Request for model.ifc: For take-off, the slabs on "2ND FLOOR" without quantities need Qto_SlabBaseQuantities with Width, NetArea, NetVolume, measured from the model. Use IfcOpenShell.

First a look at what the model holds.

```python
import ifcopenshell
import ifcopenshell.util.element
import ifcopenshell.util.unit

model = ifcopenshell.open("model.ifc")
print(model.schema)
for unit_type in ("LENGTHUNIT", "AREAUNIT", "VOLUMEUNIT"):
    print(unit_type, ifcopenshell.util.unit.calculate_unit_scale(model, unit_type))
storey = next(s for s in model.by_type("IfcBuildingStorey") if s.Name == "2ND FLOOR")
slabs = [e for e in ifcopenshell.util.element.get_decomposition(storey) if e.is_a("IfcSlab")]
for e in sorted(slabs, key=lambda e: e.id()):
    print(e.id(), e.is_a(), e.Name, list(ifcopenshell.util.element.get_psets(e, qtos_only=True)), sep=" | ")
```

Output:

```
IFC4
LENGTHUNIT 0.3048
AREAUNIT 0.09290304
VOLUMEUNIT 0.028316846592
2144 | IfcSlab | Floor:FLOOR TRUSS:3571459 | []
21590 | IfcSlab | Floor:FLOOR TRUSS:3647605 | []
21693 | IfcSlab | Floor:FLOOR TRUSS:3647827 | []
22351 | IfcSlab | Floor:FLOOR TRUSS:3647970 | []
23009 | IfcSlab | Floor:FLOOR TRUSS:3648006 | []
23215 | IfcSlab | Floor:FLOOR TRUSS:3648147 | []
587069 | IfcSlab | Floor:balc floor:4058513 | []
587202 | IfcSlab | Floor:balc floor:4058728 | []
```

```python
import ifcopenshell
import ifcopenshell.api.pset
import ifcopenshell.geom
import ifcopenshell.util.element
import ifcopenshell.util.shape
import ifcopenshell.util.unit

model = ifcopenshell.open("model.ifc")
unit_scale = ifcopenshell.util.unit.calculate_unit_scale(model)
area_scale = ifcopenshell.util.unit.calculate_unit_scale(model, "AREAUNIT")
volume_scale = ifcopenshell.util.unit.calculate_unit_scale(model, "VOLUMEUNIT")
settings = ifcopenshell.geom.settings()

storey = next(s for s in model.by_type("IfcBuildingStorey") if s.Name == "2ND FLOOR")
slabs = [e for e in ifcopenshell.util.element.get_decomposition(storey) if e.is_a("IfcSlab")]

for e in sorted(slabs, key=lambda e: e.id()):
    if ifcopenshell.util.element.get_psets(e, qtos_only=True, should_inherit=False):
        continue
    # Geometry comes back in metres, in the element's own axes.
    shape = ifcopenshell.geom.create_shape(settings, e)
    values = {
        "Width": ifcopenshell.util.shape.get_z(shape.geometry) / unit_scale,
        "NetArea": ifcopenshell.util.shape.get_footprint_area(shape.geometry) / area_scale,
        "NetVolume": ifcopenshell.util.shape.get_volume(shape.geometry) / volume_scale,
    }
    qto = ifcopenshell.api.pset.add_qto(model, product=e, name="Qto_SlabBaseQuantities")
    ifcopenshell.api.pset.edit_qto(model, qto=qto, properties=values)
    print(e.id(), {k: round(v, 3) for k, v in values.items()})

model.write("model_rev.ifc")
```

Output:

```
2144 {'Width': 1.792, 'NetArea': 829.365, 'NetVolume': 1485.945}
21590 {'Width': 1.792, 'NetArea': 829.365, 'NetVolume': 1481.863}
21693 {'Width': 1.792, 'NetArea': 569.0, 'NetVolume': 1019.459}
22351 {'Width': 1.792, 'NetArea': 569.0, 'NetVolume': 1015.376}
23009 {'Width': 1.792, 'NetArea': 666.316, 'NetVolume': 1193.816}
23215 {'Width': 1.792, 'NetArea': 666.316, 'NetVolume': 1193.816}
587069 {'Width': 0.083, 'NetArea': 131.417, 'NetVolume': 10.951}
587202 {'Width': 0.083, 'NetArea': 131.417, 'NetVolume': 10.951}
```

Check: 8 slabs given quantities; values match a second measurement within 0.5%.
